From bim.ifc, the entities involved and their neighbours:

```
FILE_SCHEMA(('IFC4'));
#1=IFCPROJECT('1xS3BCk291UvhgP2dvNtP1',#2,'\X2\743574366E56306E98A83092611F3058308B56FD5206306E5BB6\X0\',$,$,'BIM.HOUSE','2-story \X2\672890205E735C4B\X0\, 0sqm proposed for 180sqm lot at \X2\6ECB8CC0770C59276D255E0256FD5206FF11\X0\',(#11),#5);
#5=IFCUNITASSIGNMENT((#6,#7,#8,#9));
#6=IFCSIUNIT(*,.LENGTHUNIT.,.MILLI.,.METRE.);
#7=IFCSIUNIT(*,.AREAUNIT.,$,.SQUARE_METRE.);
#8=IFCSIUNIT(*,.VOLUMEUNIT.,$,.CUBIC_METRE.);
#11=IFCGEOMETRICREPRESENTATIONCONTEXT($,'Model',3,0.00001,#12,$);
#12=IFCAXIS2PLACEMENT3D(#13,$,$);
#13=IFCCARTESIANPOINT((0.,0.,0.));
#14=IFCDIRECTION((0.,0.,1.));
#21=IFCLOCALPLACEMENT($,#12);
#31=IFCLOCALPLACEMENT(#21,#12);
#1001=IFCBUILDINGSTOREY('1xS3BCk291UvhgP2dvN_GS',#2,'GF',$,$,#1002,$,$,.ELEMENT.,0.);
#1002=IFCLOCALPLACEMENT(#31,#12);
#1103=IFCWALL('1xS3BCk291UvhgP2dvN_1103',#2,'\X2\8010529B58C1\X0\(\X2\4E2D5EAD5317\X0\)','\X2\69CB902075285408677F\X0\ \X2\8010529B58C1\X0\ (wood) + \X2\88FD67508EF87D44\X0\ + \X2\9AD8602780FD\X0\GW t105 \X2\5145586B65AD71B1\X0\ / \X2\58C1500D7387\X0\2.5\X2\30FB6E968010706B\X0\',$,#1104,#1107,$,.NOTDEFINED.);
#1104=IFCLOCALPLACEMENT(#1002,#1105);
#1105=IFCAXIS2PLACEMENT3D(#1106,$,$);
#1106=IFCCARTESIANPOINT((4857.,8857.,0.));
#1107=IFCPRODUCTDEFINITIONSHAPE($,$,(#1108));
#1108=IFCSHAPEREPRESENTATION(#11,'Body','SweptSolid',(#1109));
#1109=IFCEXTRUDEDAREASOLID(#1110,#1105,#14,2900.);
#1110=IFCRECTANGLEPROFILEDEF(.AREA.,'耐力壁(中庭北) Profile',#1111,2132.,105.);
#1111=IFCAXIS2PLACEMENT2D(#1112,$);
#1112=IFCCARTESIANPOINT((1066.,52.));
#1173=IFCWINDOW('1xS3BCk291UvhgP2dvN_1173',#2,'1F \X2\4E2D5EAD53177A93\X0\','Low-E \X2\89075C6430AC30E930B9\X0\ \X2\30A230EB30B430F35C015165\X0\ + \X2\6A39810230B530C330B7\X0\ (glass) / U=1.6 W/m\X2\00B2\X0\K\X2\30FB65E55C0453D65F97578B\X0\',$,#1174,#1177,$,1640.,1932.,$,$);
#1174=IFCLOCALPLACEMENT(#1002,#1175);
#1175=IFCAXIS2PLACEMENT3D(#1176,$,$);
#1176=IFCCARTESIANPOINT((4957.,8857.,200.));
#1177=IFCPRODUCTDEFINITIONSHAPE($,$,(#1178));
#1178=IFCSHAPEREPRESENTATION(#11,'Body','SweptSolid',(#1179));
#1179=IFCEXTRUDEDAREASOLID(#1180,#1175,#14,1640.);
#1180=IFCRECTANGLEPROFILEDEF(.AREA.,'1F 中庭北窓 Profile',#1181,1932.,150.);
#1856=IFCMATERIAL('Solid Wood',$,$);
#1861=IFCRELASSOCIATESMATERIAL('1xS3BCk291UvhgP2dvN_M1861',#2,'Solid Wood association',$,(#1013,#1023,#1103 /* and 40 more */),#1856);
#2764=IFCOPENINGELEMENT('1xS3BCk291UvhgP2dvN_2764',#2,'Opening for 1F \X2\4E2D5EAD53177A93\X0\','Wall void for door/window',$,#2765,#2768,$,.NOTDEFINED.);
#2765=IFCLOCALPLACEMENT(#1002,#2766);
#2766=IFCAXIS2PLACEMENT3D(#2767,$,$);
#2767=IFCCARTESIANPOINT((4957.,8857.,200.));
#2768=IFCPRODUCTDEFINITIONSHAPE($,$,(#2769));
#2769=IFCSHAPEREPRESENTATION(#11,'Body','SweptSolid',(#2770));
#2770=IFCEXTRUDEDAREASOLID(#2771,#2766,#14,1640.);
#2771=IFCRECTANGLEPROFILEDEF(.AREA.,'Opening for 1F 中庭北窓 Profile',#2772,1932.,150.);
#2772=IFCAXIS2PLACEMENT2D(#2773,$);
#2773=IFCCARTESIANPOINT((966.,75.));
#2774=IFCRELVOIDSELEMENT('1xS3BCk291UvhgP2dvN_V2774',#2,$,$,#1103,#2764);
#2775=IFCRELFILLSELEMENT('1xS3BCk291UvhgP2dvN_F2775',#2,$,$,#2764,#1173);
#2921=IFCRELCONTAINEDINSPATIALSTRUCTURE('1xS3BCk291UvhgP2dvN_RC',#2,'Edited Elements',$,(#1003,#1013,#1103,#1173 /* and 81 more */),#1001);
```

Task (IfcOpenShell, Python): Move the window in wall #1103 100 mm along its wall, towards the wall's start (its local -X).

```python
import ifcopenshell
import ifcopenshell.api.geometry
import ifcopenshell.util.placement

model = ifcopenshell.open("bim.ifc")

window = model.by_guid("1xS3BCk291UvhgP2dvN_1173")
opening = window.FillsVoids[0].RelatingOpeningElement
wall = opening.VoidsElements[0].RelatingBuildingElement

wall_matrix = ifcopenshell.util.placement.get_local_placement(wall.ObjectPlacement)
shift = wall_matrix[:3, 0] * -100.0
before = ifcopenshell.util.placement.get_local_placement(window.ObjectPlacement)[:3, 3].copy()

# The window is not placed relative to its opening, so move both.
for product in (opening, window):
    matrix = ifcopenshell.util.placement.get_local_placement(product.ObjectPlacement)
    matrix[:3, 3] += shift
    ifcopenshell.api.geometry.edit_object_placement(model, product=product, matrix=matrix, is_si=False)

after = ifcopenshell.util.placement.get_local_placement(window.ObjectPlacement)[:3, 3]
print("window moved by", (after - before).round(3) + 0.0)

model.write("bim_edited.ifc")
```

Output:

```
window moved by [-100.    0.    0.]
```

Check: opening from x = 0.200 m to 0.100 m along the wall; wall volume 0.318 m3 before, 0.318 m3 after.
